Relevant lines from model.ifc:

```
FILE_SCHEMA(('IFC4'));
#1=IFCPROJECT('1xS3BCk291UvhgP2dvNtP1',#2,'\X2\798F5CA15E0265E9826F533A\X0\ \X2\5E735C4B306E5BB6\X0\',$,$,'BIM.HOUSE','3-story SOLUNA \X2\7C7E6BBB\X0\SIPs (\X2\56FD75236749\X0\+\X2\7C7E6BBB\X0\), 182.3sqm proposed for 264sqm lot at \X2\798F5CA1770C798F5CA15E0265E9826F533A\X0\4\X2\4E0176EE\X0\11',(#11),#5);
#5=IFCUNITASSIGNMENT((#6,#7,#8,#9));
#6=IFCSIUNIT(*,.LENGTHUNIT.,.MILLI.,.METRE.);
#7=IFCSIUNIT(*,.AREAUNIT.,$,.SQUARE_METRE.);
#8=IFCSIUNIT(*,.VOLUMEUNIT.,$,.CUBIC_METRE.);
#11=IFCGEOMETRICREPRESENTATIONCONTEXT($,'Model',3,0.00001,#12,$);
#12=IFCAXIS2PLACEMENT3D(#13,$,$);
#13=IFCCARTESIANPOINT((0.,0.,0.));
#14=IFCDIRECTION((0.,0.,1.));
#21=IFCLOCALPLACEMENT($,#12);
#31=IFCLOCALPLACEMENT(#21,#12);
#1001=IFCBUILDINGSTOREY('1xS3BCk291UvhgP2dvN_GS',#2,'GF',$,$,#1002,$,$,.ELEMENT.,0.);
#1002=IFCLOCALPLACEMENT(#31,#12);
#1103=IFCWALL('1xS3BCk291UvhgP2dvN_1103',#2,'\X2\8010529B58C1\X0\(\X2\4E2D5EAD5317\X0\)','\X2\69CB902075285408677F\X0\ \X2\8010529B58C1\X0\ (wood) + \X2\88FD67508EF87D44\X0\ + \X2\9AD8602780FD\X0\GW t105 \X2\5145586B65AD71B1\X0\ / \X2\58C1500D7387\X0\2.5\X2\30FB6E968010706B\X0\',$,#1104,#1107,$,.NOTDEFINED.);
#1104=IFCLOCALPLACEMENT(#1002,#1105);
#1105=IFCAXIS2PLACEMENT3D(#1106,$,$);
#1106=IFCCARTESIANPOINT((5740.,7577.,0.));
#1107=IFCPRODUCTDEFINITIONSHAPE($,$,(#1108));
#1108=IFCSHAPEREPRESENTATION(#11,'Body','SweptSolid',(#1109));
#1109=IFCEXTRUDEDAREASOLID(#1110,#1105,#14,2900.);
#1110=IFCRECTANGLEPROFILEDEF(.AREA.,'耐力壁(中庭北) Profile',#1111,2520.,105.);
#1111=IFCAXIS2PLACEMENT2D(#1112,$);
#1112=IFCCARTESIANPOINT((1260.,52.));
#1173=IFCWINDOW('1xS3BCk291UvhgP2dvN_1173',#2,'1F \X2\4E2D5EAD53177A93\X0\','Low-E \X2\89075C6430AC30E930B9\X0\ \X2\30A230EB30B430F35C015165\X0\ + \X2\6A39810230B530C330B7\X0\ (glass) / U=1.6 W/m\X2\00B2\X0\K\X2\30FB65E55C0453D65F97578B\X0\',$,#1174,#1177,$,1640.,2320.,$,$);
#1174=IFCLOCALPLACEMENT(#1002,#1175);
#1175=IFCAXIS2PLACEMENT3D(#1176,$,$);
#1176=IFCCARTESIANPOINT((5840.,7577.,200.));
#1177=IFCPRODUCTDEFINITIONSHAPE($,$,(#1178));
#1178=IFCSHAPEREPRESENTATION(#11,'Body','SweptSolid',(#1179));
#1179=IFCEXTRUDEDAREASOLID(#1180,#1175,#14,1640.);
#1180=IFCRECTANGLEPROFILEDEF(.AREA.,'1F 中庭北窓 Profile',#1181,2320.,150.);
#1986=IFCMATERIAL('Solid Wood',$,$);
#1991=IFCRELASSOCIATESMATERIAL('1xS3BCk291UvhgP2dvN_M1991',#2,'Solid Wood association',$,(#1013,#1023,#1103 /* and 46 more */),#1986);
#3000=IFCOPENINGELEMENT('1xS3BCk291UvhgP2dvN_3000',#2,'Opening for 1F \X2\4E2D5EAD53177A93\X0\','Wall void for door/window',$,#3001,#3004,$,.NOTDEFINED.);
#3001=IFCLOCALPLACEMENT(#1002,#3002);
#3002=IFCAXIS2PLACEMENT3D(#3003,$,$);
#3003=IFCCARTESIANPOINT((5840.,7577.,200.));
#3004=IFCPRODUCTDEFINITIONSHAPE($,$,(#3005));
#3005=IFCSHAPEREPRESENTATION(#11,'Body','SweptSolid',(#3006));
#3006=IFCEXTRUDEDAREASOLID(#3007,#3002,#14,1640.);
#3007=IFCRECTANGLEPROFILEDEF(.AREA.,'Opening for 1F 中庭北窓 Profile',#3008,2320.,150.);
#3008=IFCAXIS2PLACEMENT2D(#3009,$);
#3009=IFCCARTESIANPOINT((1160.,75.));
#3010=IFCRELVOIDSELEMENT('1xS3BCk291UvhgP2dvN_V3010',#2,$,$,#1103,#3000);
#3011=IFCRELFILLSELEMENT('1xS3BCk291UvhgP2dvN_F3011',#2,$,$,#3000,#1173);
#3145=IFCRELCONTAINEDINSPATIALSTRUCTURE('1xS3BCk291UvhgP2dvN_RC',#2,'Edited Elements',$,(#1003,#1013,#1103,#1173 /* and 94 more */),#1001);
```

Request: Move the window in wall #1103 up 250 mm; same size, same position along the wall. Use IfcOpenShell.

```python
import numpy as np
import ifcopenshell
import ifcopenshell.api.geometry
import ifcopenshell.util.placement
import ifcopenshell.util.unit

model = ifcopenshell.open("model.ifc")
unit_scale = ifcopenshell.util.unit.calculate_unit_scale(model)

window = model.by_id(1173)
opening = window.FillsVoids[0].RelatingOpeningElement
dz = 250.0

shift = np.array([0.0, 0.0, dz])
# The window is not placed relative to its opening, so move both.
for product in (opening, window):
    matrix = ifcopenshell.util.placement.get_local_placement(product.ObjectPlacement)
    matrix[:3, 3] += shift
    ifcopenshell.api.geometry.edit_object_placement(model, product=product, matrix=matrix, is_si=False)

print(f"moved by {dz * unit_scale:+.3f} m")

model.write("model-out.ifc")
```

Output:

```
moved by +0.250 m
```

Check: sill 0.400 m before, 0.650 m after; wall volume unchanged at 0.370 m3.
